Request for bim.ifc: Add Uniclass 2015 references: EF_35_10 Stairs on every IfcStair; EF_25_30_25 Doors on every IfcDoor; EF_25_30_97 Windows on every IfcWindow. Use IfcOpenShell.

First a look at what the model holds.

```python
import ifcopenshell

model = ifcopenshell.open("bim.ifc")
print(model.schema)
print("classifications:", [c.Name for c in model.by_type("IfcClassification")])
for ifc_class in ("IfcDoor", "IfcRoof", "IfcStair", "IfcWall", "IfcWindow"):
    print(ifc_class, len(model.by_type(ifc_class)))
```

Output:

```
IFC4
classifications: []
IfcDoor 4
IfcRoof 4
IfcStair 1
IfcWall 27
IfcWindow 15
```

```python
import ifcopenshell
import ifcopenshell.api.classification

model = ifcopenshell.open("bim.ifc")

system = ifcopenshell.api.classification.add_classification(model, classification="Uniclass 2015")

codes = {
    "IfcStair": ("EF_35_10", "Stairs"),
    "IfcDoor": ("EF_25_30_25", "Doors"),
    "IfcWindow": ("EF_25_30_97", "Windows"),
}
for ifc_class, (code, name) in codes.items():
    products = model.by_type(ifc_class)
    ifcopenshell.api.classification.add_reference(
        model, products=products, classification=system, identification=code, name=name
    )
    print(code, len(products))

model.write("bim_rev.ifc")
```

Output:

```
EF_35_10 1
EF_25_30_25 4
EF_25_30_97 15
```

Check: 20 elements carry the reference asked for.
